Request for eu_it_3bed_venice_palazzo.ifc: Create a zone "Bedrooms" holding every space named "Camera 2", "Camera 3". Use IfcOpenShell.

First a look at what the model holds.

```python
import ifcopenshell

model = ifcopenshell.open("eu_it_3bed_venice_palazzo.ifc")
print(model.schema)
seen = {}
for space in model.by_type("IfcSpace"):
    seen[space.LongName] = seen.get(space.LongName, 0) + 1
for name, count in sorted(seen.items(), key=str):
    print(count, "x", name)
print("zones:", [z.Name for z in model.by_type("IfcZone")][:20])
```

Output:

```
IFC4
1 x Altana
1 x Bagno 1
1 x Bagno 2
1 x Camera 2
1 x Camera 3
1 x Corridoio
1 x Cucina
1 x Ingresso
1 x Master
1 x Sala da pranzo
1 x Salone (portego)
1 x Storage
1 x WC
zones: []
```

```python
import ifcopenshell
import ifcopenshell.api.group
import ifcopenshell.api.root

model = ifcopenshell.open("eu_it_3bed_venice_palazzo.ifc")

names = {"Camera 2", "Camera 3"}
spaces = [s for s in model.by_type("IfcSpace") if s.LongName in names]

zone = ifcopenshell.api.root.create_entity(model, ifc_class="IfcZone", name="Bedrooms")
ifcopenshell.api.group.assign_group(model, products=spaces, group=zone)
print(len(spaces), "spaces in", zone.Name)

model.write("eu_it_3bed_venice_palazzo_rev.ifc")
```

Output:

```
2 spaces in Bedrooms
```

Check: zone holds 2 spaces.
